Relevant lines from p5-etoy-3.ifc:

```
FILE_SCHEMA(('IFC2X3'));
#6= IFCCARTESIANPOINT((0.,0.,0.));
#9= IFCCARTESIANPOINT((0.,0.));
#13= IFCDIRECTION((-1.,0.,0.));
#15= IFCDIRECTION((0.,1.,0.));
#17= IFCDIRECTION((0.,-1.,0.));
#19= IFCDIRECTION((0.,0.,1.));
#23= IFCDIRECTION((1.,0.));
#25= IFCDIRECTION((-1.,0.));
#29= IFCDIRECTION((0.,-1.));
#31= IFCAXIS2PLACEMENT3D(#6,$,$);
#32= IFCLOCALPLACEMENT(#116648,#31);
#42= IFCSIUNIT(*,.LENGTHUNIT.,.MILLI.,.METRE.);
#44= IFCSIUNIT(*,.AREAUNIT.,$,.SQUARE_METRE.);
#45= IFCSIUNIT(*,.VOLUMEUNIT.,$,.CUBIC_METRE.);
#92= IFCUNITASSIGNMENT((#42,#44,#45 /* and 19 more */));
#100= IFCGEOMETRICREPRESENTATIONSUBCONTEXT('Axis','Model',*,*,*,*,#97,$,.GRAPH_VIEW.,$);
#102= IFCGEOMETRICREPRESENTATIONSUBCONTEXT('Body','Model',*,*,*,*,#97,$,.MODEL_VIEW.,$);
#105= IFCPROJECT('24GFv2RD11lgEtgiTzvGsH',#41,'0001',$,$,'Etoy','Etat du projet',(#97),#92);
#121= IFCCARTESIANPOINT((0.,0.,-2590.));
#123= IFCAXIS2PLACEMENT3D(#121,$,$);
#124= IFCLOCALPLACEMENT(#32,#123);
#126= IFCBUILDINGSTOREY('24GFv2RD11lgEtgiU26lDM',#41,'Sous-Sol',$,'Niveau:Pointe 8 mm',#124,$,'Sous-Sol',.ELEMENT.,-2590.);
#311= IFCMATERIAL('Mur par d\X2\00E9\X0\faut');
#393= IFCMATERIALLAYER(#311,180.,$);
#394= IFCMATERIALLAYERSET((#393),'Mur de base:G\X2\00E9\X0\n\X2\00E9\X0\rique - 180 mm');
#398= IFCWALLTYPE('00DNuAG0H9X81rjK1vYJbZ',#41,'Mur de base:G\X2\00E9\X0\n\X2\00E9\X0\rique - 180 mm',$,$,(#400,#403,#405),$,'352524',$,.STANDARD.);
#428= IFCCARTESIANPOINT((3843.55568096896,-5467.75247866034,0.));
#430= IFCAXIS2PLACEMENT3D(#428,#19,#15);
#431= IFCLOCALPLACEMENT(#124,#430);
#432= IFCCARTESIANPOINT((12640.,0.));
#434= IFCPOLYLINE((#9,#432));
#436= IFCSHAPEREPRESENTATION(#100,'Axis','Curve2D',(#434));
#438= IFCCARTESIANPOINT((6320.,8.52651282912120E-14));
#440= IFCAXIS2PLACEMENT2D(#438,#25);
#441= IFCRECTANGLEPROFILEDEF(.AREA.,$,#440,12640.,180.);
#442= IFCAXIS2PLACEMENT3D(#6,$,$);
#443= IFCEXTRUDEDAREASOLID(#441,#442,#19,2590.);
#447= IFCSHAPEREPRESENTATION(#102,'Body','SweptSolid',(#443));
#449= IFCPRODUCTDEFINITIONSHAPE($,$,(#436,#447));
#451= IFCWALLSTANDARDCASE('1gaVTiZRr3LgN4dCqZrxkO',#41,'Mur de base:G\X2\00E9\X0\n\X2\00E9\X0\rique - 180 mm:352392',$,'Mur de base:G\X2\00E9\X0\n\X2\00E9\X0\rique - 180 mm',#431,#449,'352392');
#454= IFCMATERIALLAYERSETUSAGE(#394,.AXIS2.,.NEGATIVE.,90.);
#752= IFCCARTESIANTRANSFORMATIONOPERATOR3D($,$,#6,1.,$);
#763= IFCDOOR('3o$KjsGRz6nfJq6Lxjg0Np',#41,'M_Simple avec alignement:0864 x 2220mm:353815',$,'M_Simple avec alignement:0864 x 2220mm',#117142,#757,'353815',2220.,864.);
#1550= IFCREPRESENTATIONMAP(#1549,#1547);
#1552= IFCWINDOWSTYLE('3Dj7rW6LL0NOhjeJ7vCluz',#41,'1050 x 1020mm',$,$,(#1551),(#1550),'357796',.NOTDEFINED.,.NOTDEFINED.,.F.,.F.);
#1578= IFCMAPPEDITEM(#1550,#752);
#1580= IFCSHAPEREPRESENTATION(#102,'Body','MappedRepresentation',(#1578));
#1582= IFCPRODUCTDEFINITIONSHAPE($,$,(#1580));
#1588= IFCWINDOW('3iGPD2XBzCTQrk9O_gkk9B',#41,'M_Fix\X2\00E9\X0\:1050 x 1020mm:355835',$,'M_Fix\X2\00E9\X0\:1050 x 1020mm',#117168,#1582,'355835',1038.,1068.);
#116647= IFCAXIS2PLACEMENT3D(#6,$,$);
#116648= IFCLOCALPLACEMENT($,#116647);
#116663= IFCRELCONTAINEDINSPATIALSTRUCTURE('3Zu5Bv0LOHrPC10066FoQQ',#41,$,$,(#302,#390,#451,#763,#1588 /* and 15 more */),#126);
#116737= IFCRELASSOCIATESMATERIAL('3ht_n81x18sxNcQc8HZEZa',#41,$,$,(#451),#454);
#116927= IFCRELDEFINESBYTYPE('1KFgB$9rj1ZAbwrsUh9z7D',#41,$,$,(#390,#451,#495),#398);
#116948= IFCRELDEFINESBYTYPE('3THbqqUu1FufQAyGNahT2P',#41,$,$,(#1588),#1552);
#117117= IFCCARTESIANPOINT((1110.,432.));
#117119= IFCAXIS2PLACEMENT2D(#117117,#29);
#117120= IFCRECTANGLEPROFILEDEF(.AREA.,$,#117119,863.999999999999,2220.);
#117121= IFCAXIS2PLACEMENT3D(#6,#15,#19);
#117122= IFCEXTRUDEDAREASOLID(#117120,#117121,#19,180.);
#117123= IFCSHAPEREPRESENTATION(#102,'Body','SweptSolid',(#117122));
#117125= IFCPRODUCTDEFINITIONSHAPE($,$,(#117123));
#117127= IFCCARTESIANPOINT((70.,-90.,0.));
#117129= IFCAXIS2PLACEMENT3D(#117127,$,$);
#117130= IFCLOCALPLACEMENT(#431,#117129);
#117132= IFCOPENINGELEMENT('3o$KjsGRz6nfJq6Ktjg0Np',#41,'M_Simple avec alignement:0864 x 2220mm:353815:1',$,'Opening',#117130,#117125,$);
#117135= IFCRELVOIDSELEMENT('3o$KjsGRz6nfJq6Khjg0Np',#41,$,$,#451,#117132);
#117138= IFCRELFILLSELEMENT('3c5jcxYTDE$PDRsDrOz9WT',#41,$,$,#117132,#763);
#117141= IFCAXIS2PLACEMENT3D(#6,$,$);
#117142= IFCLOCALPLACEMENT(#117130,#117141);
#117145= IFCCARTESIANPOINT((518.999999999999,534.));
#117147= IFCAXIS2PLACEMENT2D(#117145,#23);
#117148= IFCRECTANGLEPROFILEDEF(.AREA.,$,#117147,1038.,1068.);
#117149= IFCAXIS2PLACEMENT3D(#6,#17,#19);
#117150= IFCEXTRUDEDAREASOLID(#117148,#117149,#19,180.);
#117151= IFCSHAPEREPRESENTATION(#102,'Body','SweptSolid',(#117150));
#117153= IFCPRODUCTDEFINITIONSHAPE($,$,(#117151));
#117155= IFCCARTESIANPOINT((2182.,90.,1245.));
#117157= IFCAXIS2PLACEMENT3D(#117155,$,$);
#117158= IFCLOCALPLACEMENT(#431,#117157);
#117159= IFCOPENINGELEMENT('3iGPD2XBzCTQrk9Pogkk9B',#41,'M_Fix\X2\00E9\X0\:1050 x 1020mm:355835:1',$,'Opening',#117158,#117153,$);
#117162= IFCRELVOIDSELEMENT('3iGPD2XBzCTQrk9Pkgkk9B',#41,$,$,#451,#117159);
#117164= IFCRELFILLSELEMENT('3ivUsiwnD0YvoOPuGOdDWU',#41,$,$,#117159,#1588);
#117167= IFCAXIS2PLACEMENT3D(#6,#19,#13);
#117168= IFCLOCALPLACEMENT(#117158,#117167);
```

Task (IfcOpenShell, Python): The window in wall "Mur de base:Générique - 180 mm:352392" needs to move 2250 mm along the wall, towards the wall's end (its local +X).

```python
import ifcopenshell
import ifcopenshell.api.geometry
import ifcopenshell.util.placement

model = ifcopenshell.open("p5-etoy-3.ifc")

window = model.by_id(1588)
opening = window.FillsVoids[0].RelatingOpeningElement
wall = opening.VoidsElements[0].RelatingBuildingElement

wall_matrix = ifcopenshell.util.placement.get_local_placement(wall.ObjectPlacement)
shift = wall_matrix[:3, 0] * 2250.0
before = ifcopenshell.util.placement.get_local_placement(window.ObjectPlacement)[:3, 3].copy()

# The window is placed relative to its opening, so it follows when the opening moves.
matrix = ifcopenshell.util.placement.get_local_placement(opening.ObjectPlacement)
matrix[:3, 3] += shift
ifcopenshell.api.geometry.edit_object_placement(
    model, product=opening, matrix=matrix, is_si=False, should_transform_children=True
)

after = ifcopenshell.util.placement.get_local_placement(window.ObjectPlacement)[:3, 3]
print("window moved by", (after - before).round(3) + 0.0)

model.write("p5-etoy-3-out.ifc")
```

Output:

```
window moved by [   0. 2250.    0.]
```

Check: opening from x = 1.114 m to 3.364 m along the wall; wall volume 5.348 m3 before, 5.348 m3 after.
